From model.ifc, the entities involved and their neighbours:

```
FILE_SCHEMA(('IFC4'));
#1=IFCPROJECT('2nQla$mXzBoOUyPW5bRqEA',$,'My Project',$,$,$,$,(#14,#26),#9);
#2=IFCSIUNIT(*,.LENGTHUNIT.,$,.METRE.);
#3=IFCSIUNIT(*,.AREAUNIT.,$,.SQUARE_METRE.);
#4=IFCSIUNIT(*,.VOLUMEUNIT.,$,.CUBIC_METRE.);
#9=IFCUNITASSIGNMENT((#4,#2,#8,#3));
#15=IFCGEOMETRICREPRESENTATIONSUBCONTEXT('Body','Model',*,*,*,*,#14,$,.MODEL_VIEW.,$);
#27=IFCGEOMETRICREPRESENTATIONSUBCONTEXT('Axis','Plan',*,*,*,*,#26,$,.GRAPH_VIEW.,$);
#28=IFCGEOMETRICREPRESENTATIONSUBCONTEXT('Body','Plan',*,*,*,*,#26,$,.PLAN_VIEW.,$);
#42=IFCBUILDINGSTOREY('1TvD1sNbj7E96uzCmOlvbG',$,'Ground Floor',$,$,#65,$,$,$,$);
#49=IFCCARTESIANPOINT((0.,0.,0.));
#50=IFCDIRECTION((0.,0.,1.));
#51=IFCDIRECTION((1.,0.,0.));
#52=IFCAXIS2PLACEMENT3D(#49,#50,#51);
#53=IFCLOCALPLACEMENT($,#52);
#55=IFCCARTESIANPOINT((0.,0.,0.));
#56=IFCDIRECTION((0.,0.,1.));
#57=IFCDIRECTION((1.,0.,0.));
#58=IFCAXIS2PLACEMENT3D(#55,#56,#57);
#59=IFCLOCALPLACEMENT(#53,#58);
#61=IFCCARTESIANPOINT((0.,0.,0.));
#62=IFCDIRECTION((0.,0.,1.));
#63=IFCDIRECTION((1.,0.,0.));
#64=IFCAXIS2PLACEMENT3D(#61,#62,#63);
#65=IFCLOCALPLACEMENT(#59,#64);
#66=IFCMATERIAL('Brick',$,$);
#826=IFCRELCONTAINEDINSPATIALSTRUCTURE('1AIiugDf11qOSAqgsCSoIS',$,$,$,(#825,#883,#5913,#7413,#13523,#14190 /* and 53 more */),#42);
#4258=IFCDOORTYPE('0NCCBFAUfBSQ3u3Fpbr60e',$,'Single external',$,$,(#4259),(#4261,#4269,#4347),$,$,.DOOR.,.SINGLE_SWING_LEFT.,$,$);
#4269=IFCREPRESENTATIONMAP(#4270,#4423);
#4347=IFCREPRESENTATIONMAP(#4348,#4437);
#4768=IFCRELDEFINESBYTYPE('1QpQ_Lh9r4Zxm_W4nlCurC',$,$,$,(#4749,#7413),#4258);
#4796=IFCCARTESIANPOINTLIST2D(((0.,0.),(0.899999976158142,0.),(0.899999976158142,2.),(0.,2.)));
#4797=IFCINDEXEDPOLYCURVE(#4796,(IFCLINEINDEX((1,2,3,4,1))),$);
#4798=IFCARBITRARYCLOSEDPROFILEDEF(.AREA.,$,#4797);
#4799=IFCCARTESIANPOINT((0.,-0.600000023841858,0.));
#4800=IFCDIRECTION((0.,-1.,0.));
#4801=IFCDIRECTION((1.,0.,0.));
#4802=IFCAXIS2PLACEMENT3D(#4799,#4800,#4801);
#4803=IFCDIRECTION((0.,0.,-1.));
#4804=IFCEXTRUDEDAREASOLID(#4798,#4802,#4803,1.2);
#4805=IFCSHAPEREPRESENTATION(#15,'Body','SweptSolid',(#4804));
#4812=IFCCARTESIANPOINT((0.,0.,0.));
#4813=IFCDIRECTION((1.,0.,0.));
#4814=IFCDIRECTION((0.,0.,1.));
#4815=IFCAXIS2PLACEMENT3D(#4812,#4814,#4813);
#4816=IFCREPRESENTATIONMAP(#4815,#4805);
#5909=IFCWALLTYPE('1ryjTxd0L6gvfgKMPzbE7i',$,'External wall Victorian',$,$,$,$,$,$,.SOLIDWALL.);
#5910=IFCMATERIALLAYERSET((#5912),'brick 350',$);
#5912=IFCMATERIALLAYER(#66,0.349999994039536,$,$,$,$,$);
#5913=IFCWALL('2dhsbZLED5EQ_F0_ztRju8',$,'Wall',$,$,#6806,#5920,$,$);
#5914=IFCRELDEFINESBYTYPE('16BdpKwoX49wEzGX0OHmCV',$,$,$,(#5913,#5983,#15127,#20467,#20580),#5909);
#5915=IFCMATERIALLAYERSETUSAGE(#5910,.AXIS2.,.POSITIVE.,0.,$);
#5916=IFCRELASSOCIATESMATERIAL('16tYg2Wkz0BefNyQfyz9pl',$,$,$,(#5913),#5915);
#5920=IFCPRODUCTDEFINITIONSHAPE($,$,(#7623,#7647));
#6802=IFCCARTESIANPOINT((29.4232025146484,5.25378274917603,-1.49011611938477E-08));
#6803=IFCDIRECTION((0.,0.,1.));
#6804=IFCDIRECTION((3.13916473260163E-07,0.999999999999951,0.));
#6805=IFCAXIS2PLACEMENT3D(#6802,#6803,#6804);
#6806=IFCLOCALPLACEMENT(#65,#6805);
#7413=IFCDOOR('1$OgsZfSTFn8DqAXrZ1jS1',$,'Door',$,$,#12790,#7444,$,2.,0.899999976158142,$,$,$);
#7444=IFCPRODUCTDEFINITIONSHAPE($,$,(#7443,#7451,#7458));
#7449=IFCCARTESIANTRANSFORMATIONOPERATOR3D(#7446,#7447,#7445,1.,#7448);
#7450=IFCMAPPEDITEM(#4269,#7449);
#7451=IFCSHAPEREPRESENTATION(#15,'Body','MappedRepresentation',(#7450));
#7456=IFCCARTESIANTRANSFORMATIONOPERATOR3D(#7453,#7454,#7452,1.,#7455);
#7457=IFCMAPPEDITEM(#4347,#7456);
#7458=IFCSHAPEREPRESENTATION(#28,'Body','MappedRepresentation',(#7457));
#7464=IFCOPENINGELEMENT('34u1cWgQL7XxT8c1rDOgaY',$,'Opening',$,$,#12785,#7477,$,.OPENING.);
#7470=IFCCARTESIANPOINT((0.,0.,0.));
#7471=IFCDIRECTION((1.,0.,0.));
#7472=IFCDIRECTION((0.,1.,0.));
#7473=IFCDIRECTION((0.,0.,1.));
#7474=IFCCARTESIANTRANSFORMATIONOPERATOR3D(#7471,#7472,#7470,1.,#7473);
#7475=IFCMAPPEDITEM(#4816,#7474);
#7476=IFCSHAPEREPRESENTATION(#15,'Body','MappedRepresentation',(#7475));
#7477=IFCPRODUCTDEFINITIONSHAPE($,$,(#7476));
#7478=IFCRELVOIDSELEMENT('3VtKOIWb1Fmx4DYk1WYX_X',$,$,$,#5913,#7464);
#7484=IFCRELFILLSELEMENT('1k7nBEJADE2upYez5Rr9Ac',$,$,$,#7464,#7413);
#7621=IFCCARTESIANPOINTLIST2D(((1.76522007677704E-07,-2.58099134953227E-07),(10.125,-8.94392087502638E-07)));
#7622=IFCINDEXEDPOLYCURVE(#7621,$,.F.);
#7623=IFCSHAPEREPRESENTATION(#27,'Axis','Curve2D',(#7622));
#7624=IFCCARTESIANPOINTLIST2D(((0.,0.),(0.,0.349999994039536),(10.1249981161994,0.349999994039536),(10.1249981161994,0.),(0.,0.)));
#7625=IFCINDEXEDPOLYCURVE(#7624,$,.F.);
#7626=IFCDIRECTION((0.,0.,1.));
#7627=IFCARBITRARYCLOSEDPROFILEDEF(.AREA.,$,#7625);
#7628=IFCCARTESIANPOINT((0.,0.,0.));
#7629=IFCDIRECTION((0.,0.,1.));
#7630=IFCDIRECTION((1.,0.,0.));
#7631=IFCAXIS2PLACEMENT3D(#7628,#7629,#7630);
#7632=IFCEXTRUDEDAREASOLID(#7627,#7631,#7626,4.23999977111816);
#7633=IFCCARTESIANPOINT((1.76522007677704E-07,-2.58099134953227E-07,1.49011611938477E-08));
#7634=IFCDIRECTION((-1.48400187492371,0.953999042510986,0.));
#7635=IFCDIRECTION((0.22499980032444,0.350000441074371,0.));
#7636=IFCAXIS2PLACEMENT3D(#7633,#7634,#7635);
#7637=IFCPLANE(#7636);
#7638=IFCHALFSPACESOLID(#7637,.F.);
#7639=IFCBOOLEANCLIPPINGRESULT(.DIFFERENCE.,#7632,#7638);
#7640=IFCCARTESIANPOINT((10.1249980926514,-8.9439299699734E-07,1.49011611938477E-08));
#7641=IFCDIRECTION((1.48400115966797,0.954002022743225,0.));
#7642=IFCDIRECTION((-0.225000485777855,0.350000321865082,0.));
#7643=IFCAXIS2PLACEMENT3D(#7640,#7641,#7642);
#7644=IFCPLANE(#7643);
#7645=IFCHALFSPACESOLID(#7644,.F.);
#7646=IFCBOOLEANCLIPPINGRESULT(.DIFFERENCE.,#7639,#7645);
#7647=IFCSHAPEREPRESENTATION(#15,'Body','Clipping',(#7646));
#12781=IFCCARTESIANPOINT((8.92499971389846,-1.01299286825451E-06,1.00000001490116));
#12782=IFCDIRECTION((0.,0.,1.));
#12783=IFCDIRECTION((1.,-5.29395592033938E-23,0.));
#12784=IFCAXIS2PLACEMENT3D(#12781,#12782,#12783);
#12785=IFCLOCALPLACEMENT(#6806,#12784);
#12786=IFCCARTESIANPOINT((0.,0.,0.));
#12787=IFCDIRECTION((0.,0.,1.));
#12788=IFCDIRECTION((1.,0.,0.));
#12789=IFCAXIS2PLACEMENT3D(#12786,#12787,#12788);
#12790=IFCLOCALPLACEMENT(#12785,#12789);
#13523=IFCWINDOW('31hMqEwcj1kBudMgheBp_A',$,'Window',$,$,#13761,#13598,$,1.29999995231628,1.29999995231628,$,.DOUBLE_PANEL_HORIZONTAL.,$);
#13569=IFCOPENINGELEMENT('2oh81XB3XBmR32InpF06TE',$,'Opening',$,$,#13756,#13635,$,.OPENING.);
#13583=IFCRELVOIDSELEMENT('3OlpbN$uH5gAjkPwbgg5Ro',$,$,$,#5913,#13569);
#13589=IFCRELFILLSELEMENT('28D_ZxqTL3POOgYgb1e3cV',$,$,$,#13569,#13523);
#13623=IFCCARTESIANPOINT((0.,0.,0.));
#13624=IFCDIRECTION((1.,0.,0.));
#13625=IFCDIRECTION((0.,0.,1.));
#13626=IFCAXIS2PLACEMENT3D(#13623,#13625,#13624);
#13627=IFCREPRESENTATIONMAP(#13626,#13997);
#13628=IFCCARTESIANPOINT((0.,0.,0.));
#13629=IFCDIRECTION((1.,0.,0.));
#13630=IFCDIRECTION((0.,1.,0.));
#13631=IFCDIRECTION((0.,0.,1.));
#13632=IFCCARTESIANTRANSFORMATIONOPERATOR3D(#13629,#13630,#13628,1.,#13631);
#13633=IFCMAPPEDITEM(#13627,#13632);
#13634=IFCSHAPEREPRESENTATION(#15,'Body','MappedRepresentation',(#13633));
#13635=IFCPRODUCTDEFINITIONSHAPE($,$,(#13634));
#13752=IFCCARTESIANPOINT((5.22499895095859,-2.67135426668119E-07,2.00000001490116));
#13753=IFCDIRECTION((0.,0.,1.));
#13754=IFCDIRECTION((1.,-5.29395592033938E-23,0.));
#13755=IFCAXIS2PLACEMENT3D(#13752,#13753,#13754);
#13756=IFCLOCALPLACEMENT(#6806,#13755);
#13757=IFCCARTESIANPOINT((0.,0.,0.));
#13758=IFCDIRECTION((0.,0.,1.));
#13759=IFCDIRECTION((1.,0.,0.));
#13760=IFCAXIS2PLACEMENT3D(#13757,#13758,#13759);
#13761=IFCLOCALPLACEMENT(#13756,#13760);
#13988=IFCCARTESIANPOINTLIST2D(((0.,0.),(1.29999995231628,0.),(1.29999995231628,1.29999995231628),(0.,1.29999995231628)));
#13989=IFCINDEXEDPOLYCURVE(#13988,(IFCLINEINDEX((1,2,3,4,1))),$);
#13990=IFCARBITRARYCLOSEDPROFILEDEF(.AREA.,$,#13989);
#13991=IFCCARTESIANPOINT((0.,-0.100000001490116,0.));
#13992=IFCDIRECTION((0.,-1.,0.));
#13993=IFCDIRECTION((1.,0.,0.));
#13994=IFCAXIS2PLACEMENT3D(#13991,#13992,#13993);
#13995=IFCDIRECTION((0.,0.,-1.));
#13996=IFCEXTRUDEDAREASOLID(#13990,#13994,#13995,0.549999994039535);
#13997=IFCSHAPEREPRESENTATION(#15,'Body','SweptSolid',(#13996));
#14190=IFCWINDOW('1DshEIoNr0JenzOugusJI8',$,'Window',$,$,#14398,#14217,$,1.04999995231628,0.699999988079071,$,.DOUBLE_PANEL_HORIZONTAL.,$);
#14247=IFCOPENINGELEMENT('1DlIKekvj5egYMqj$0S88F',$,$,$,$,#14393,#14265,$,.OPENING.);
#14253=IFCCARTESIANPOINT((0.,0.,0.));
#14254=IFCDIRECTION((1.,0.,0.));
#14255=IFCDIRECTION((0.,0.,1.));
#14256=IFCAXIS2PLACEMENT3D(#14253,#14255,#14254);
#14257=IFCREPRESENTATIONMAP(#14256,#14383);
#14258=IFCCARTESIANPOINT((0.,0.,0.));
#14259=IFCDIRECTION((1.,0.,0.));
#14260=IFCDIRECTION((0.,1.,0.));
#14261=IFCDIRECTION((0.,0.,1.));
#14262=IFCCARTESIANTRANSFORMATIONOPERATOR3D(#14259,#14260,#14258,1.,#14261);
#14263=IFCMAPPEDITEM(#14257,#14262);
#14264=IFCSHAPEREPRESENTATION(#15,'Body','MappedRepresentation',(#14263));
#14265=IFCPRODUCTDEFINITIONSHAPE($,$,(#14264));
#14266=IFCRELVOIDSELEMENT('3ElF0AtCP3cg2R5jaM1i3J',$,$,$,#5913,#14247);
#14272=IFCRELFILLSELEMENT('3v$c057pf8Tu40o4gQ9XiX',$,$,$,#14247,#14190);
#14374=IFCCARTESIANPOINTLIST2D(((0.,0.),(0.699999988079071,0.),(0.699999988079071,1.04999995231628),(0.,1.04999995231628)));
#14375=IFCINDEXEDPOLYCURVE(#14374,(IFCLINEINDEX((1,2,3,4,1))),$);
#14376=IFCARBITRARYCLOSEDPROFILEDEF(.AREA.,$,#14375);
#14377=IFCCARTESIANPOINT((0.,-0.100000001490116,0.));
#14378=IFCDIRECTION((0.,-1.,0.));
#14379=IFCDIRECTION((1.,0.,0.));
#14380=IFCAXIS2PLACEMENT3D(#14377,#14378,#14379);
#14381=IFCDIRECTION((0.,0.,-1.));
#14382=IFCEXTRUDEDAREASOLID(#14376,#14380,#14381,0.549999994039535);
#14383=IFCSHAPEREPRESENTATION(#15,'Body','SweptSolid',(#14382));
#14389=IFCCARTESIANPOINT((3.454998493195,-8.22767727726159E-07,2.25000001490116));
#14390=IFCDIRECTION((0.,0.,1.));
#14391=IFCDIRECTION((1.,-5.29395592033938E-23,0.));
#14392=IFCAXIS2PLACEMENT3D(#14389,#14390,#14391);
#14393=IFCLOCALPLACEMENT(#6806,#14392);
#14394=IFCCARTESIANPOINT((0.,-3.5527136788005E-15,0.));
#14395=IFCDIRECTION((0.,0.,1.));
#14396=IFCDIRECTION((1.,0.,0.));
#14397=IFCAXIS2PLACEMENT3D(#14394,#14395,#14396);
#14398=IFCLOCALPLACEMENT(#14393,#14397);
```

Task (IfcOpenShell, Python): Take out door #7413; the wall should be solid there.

```python
import ifcopenshell
import ifcopenshell.api.feature
import ifcopenshell.api.root
import ifcopenshell.geom
import ifcopenshell.util.shape

model = ifcopenshell.open("model.ifc")
settings = ifcopenshell.geom.settings()


def volume(element):
    """Net volume in cubic metres, openings subtracted."""
    shape = ifcopenshell.geom.create_shape(settings, element)
    return ifcopenshell.util.shape.get_volume(shape.geometry)


door = model.by_guid("1$OgsZfSTFn8DqAXrZ1jS1")
opening = door.FillsVoids[0].RelatingOpeningElement
wall = opening.VoidsElements[0].RelatingBuildingElement
before = volume(wall)

ifcopenshell.api.root.remove_product(model, product=door)
ifcopenshell.api.feature.remove_feature(model, feature=opening)

after = volume(wall)

print(f"wall volume {before:.3f} -> {after:.3f} m3")

model.write("model_edited.ifc")
```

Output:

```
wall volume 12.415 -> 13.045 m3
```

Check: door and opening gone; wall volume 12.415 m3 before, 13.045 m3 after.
